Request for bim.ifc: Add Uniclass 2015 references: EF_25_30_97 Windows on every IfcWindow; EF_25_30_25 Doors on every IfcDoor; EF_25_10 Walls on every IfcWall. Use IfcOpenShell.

First a look at what the model holds.

```python
import ifcopenshell

model = ifcopenshell.open("bim.ifc")
print(model.schema)
print("classifications:", [c.Name for c in model.by_type("IfcClassification")])
for ifc_class in ("IfcDoor", "IfcRoof", "IfcStair", "IfcWall", "IfcWindow"):
    print(ifc_class, len(model.by_type(ifc_class)))
```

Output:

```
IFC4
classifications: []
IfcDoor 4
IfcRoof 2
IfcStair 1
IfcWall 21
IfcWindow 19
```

```python
import ifcopenshell
import ifcopenshell.api.classification

model = ifcopenshell.open("bim.ifc")

system = ifcopenshell.api.classification.add_classification(model, classification="Uniclass 2015")

codes = {
    "IfcWindow": ("EF_25_30_97", "Windows"),
    "IfcDoor": ("EF_25_30_25", "Doors"),
    "IfcWall": ("EF_25_10", "Walls"),
}
for ifc_class, (code, name) in codes.items():
    products = model.by_type(ifc_class)
    ifcopenshell.api.classification.add_reference(
        model, products=products, classification=system, identification=code, name=name
    )
    print(code, len(products))

model.write("bim_rev.ifc")
```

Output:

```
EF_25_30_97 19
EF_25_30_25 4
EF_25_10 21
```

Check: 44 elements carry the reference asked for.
